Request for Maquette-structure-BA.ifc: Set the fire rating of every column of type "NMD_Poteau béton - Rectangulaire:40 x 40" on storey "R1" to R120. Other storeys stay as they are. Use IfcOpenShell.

First a look at what the model holds.

```python
import ifcopenshell
import ifcopenshell.util.element

model = ifcopenshell.open("Maquette-structure-BA.ifc")
print(model.schema)
storey = next(s for s in model.by_type("IfcBuildingStorey") if s.Name == "R1")
columns = [e for e in ifcopenshell.util.element.get_decomposition(storey) if e.is_a("IfcColumn")]
seen = {}
for e in columns:
    element_type = ifcopenshell.util.element.get_type(e)
    key = (element_type.Name if element_type != e and element_type else None, ifcopenshell.util.element.get_pset(e, "Pset_ColumnCommon", "FireRating"))
    seen[key] = seen.get(key, 0) + 1
for (name, value), count in sorted(seen.items(), key=str):
    print(count, "x", name, "|", value)
```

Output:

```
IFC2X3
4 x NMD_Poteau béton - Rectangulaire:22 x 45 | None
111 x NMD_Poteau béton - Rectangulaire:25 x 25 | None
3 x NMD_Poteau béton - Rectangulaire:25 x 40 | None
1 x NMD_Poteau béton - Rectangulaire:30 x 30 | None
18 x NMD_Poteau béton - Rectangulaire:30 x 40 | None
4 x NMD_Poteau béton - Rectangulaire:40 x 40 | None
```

```python
import ifcopenshell
import ifcopenshell.api.pset
import ifcopenshell.util.element

model = ifcopenshell.open("Maquette-structure-BA.ifc")

storey = next(s for s in model.by_type("IfcBuildingStorey") if s.Name == "R1")
columns = [e for e in ifcopenshell.util.element.get_decomposition(storey) if e.is_a("IfcColumn")]

count = 0
for e in columns:
    element_type = ifcopenshell.util.element.get_type(e)
    if element_type in (None, e) or element_type.Name != "NMD_Poteau béton - Rectangulaire:40 x 40":
        continue
    # add_pset returns the element's existing set when there is one.
    pset = ifcopenshell.api.pset.add_pset(model, product=e, name="Pset_ColumnCommon")
    ifcopenshell.api.pset.edit_pset(model, pset=pset, properties={"FireRating": "R120"})
    count += 1

print(count, "columns updated")

model.write("Maquette-structure-BA_updated.ifc")
```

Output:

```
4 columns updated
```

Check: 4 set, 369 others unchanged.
